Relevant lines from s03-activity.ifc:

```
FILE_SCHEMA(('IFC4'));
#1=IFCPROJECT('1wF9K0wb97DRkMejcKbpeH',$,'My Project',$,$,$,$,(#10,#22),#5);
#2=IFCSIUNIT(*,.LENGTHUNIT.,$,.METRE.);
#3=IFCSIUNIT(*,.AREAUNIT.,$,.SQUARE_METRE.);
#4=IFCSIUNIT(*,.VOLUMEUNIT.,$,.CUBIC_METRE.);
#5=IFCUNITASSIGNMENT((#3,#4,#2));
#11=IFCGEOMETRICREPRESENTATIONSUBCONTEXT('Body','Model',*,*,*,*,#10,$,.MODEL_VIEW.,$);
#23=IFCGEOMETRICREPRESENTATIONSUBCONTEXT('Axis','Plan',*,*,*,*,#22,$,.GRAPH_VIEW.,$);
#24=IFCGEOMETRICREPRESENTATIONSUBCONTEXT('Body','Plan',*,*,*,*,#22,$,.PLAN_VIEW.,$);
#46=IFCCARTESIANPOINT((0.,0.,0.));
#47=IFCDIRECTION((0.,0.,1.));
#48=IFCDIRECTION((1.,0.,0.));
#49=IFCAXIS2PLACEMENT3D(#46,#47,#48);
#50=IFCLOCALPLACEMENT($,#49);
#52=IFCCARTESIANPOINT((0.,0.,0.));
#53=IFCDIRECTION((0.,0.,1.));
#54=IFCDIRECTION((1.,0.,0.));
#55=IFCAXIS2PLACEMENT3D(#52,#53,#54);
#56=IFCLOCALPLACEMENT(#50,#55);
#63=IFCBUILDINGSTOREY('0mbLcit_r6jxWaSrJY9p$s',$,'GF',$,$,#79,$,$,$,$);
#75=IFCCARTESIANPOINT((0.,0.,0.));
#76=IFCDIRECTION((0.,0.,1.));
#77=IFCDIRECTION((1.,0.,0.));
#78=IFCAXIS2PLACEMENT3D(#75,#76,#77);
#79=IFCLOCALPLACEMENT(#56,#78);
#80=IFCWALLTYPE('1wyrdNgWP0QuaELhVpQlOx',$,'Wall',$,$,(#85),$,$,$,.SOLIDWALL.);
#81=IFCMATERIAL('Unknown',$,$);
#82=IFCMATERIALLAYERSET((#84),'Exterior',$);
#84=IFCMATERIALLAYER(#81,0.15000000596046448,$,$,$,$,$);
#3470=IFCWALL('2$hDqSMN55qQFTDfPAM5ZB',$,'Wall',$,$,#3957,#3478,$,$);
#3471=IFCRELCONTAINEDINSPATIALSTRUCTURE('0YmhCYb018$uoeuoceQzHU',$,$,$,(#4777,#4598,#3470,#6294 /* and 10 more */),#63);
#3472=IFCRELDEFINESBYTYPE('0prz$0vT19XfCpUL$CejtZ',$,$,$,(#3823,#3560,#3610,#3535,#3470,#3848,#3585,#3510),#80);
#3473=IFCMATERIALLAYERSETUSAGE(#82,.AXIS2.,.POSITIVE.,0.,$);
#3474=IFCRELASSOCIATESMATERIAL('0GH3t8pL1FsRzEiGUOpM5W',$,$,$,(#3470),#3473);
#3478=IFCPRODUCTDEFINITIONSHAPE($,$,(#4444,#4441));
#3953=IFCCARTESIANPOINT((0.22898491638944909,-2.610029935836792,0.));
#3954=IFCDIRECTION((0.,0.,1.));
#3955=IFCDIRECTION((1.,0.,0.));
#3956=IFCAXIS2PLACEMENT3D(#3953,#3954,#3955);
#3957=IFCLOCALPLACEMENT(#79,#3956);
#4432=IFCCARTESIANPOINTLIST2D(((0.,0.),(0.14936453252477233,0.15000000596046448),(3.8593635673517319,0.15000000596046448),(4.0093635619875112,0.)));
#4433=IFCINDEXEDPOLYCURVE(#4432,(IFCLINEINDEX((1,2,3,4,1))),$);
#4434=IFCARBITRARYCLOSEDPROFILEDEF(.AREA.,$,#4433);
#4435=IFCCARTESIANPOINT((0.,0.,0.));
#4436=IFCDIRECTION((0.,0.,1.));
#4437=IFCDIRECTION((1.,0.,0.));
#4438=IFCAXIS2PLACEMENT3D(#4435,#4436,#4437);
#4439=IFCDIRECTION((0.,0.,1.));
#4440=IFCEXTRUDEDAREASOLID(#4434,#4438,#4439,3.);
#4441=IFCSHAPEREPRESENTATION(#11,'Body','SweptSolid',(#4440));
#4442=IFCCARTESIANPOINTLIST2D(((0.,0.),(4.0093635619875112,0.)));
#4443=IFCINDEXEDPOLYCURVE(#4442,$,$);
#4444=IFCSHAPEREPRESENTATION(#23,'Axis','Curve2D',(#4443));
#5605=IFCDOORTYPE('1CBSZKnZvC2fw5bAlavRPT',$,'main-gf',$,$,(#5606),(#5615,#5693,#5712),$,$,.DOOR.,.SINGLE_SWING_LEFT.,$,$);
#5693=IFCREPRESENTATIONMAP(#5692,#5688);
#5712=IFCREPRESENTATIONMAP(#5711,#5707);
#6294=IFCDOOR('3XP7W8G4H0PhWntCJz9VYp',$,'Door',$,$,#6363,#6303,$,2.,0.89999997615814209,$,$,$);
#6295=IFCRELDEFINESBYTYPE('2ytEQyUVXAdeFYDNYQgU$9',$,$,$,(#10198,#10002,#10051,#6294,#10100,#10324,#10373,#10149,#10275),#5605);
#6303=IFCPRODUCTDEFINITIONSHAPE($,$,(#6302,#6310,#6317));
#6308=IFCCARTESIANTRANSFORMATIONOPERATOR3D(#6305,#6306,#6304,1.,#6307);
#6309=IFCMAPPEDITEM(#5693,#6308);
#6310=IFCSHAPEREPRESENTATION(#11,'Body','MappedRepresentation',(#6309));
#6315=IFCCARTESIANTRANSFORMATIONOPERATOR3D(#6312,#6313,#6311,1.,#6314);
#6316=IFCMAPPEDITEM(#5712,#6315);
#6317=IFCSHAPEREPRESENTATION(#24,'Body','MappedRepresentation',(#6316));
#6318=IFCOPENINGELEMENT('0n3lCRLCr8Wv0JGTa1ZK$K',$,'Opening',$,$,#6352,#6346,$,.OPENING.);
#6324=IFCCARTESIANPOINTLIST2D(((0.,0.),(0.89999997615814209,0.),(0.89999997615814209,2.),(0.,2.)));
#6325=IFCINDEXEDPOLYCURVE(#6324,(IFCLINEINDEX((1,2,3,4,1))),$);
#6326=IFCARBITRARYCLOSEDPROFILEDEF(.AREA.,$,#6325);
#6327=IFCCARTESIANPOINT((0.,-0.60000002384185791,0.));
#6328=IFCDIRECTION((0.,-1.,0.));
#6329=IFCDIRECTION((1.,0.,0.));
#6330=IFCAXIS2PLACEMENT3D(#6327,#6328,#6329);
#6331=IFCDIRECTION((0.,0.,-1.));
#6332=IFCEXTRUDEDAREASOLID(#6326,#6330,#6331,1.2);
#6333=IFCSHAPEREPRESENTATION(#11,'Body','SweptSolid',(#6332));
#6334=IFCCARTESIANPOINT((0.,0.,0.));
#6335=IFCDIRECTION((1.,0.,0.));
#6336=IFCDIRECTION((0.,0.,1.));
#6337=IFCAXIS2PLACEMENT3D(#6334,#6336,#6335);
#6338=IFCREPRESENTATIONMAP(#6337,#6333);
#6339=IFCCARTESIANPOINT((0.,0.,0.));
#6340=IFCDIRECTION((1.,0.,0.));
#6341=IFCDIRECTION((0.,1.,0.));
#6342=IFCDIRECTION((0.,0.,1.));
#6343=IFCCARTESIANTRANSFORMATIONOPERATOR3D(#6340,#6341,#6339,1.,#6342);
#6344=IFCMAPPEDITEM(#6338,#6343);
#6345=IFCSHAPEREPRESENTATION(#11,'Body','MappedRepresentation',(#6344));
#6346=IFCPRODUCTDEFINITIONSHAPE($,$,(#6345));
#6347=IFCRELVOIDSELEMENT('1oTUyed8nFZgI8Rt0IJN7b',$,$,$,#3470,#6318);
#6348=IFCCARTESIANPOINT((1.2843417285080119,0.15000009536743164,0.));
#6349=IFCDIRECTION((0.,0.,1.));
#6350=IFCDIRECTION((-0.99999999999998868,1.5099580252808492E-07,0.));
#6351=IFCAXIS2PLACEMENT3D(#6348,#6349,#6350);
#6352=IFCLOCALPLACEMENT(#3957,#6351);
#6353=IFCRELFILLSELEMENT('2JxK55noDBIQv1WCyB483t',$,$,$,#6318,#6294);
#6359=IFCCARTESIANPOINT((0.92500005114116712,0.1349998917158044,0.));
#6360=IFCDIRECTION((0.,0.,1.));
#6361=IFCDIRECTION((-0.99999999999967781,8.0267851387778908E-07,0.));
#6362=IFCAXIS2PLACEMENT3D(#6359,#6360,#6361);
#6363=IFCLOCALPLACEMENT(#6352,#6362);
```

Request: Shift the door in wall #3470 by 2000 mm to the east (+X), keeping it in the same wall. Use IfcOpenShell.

```python
import ifcopenshell
import ifcopenshell.api.geometry
import ifcopenshell.util.placement
import ifcopenshell.util.unit

model = ifcopenshell.open("s03-activity.ifc")
unit_scale = ifcopenshell.util.unit.calculate_unit_scale(model)

door = model.by_guid("3XP7W8G4H0PhWntCJz9VYp")
opening = door.FillsVoids[0].RelatingOpeningElement
wall = opening.VoidsElements[0].RelatingBuildingElement

wall_matrix = ifcopenshell.util.placement.get_local_placement(wall.ObjectPlacement)
shift = wall_matrix[:3, 0] * 2 / unit_scale
before = ifcopenshell.util.placement.get_local_placement(door.ObjectPlacement)[:3, 3].copy()

# The door is placed relative to its opening, so it follows when the opening moves.
matrix = ifcopenshell.util.placement.get_local_placement(opening.ObjectPlacement)
matrix[:3, 3] += shift
ifcopenshell.api.geometry.edit_object_placement(
    model, product=opening, matrix=matrix, is_si=False, should_transform_children=True
)

after = ifcopenshell.util.placement.get_local_placement(door.ObjectPlacement)[:3, 3]
print("door moved by", (after - before).round(3) + 0.0)

model.write("s03-activity_edited.ifc")
```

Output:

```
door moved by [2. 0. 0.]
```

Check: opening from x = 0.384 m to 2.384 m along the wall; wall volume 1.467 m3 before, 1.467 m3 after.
